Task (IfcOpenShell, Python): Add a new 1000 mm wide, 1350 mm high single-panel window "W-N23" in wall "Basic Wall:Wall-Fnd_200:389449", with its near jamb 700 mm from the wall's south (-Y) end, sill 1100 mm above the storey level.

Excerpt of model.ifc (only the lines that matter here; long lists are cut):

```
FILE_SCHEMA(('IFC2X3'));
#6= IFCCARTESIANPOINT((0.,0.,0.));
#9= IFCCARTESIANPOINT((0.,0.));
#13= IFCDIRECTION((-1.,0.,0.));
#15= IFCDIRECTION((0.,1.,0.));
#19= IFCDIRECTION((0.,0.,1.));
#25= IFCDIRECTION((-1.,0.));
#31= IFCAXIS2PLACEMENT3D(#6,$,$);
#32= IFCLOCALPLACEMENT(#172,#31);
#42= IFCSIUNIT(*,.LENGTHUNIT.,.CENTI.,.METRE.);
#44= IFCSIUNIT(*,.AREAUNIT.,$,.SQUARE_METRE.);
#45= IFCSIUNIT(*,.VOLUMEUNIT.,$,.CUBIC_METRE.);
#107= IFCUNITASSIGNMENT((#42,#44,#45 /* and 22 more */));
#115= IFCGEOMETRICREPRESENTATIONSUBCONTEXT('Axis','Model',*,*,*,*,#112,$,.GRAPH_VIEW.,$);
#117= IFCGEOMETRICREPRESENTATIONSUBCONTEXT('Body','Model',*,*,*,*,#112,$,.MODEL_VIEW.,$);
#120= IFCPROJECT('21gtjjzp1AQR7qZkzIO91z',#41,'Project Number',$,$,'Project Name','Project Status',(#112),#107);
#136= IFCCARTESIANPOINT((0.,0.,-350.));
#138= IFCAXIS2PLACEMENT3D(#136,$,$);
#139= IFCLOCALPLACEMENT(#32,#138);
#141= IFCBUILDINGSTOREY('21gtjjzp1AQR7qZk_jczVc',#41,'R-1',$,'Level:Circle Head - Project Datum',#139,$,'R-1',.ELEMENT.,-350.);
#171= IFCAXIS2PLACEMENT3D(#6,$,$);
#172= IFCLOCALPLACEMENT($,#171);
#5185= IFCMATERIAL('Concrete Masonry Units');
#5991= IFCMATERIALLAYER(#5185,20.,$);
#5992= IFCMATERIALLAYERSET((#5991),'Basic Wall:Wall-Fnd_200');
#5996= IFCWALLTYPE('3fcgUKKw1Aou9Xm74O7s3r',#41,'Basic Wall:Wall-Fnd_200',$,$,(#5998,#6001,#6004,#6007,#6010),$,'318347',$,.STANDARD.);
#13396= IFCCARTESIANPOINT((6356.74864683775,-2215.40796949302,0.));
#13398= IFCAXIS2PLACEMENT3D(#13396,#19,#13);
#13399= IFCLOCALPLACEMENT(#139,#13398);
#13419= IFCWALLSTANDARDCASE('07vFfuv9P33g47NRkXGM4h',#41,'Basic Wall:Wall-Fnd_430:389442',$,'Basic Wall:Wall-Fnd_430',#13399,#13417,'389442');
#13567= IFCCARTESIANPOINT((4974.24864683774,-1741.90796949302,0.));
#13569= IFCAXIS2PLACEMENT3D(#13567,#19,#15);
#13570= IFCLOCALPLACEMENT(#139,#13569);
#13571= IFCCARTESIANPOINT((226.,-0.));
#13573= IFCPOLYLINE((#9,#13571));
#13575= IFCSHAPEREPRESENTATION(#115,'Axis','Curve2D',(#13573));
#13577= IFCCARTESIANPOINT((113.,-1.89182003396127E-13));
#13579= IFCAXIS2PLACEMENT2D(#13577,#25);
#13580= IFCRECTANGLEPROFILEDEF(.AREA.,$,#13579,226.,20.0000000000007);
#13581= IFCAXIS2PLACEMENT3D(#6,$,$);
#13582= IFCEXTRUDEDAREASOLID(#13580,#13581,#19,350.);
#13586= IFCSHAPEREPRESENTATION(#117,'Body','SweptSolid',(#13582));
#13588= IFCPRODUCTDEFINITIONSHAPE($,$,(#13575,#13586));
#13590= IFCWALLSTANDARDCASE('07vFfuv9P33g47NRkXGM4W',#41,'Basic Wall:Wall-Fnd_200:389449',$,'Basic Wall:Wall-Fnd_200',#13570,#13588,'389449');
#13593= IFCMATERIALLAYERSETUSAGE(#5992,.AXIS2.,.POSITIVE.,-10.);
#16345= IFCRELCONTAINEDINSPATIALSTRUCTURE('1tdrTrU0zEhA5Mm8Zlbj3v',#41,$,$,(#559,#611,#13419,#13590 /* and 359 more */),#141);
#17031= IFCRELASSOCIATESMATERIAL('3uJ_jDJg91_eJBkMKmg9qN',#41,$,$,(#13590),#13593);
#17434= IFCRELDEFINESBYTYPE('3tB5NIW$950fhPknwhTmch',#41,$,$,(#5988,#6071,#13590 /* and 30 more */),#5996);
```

```python
import numpy as np
import ifcopenshell
import ifcopenshell.api.feature
import ifcopenshell.api.geometry
import ifcopenshell.api.root
import ifcopenshell.api.spatial
import ifcopenshell.api.type
import ifcopenshell.geom
import ifcopenshell.util.element
import ifcopenshell.util.placement
import ifcopenshell.util.representation
import ifcopenshell.util.shape
import ifcopenshell.util.unit

model = ifcopenshell.open("model.ifc")
unit_scale = ifcopenshell.util.unit.calculate_unit_scale(model)
settings = ifcopenshell.geom.settings()


def volume(element):
    """Net volume in cubic metres, openings subtracted."""
    shape = ifcopenshell.geom.create_shape(settings, element)
    return ifcopenshell.util.shape.get_volume(shape.geometry)


wall = model.by_guid("07vFfuv9P33g47NRkXGM4W")
storey = ifcopenshell.util.element.get_container(wall, ifc_class="IfcBuildingStorey")
context = ifcopenshell.util.representation.get_context(model, "Model", "Body", "MODEL_VIEW")
before = volume(wall)

width, height, from_end, sill = 1, 1.35, 0.7, 1.1  # metres

# The wall runs along its own X axis, and the end named is its -X end.
wall_shape = ifcopenshell.geom.create_shape(settings, wall)
x, y, z = ifcopenshell.util.shape.get_vertices(wall_shape.geometry).T
start = x.min() + from_end
face, thickness = float(y.min()), float(y.max() - y.min())
wall_matrix = ifcopenshell.util.placement.get_local_placement(wall.ObjectPlacement)
level = ifcopenshell.util.placement.get_local_placement(storey.ObjectPlacement)[2, 3]


def in_wall(x, y):
    """Placement at x, y metres in the wall's axes, at sill height."""
    matrix = wall_matrix.copy()
    matrix[:, 3] = wall_matrix @ np.array([x / unit_scale, y / unit_scale, 0.0, 1.0])
    matrix[2, 3] = level + sill / unit_scale
    return matrix


# Opening: a box that overshoots both wall faces by 50 mm.
opening = ifcopenshell.api.root.create_entity(model, ifc_class="IfcOpeningElement")
box = ifcopenshell.api.geometry.add_wall_representation(
    model, context=context, length=width, height=height, thickness=thickness + 0.1
)
ifcopenshell.api.geometry.assign_representation(model, product=opening, representation=box)
ifcopenshell.api.geometry.edit_object_placement(model, product=opening, matrix=in_wall(start, face - 0.05), is_si=False)
ifcopenshell.api.feature.add_feature(model, feature=opening, element=wall)

window = ifcopenshell.api.root.create_entity(model, ifc_class="IfcWindow", name="W-N23")
window.OverallWidth, window.OverallHeight = width / unit_scale, height / unit_scale
body = ifcopenshell.api.geometry.add_window_representation(
    model,
    context=context,
    overall_width=window.OverallWidth,
    overall_height=window.OverallHeight,
    partition_type="SINGLE_PANEL",
)
ifcopenshell.api.geometry.assign_representation(model, product=window, representation=body)
ifcopenshell.api.spatial.assign_container(model, products=[window], relating_structure=storey)
fills = ifcopenshell.api.feature.add_filling(model, opening=opening, element=window)
fills.OwnerHistory = window.OwnerHistory  # required in IFC2X3

# IFC2X3 keeps the operation on the window style.
style = ifcopenshell.api.root.create_entity(model, ifc_class="IfcWindowStyle", name="W-N23")
style.OperationType, style.ConstructionType = "SINGLE_PANEL", "NOTDEFINED"
style.ParameterTakesPrecedence = style.Sizeable = False
ifcopenshell.api.type.assign_type(model, related_objects=[window], relating_type=style)

# Centre the window in the wall's thickness.
ifcopenshell.api.geometry.edit_object_placement(model, product=window, matrix=in_wall(start, face), is_si=False)
window_shape = ifcopenshell.geom.create_shape(settings, window)
depth = ifcopenshell.util.shape.get_vertices(window_shape.geometry)[:, 1]
offset = face + thickness / 2 - (depth.min() + depth.max()) / 2
ifcopenshell.api.geometry.edit_object_placement(model, product=window, matrix=in_wall(start, offset), is_si=False)

after = volume(wall)

print(f"wall volume {before:.3f} -> {after:.3f} m3")

model.write("model_updated.ifc")
```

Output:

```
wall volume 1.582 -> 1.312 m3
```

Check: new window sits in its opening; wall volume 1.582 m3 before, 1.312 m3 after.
